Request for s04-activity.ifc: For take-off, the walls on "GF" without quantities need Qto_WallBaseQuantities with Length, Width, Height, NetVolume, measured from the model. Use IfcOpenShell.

First a look at what the model holds.

```python
import ifcopenshell
import ifcopenshell.util.element
import ifcopenshell.util.unit

model = ifcopenshell.open("s04-activity.ifc")
print(model.schema)
for unit_type in ("LENGTHUNIT", "AREAUNIT", "VOLUMEUNIT"):
    print(unit_type, ifcopenshell.util.unit.calculate_unit_scale(model, unit_type))
storey = next(s for s in model.by_type("IfcBuildingStorey") if s.Name == "GF")
walls = [e for e in ifcopenshell.util.element.get_decomposition(storey) if e.is_a("IfcWall")]
for e in sorted(walls, key=lambda e: e.id()):
    print(e.id(), e.is_a(), e.Name, list(ifcopenshell.util.element.get_psets(e, qtos_only=True)), sep=" | ")
```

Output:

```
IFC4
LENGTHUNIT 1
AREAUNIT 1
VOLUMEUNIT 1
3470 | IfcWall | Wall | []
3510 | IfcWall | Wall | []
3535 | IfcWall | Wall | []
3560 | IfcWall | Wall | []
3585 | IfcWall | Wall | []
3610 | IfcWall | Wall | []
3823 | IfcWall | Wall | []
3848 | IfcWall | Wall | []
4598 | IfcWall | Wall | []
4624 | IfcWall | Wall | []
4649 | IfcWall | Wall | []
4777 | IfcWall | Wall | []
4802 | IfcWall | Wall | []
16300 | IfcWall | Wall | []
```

```python
import ifcopenshell
import ifcopenshell.api.pset
import ifcopenshell.geom
import ifcopenshell.util.element
import ifcopenshell.util.shape
import ifcopenshell.util.unit

model = ifcopenshell.open("s04-activity.ifc")
unit_scale = ifcopenshell.util.unit.calculate_unit_scale(model)
volume_scale = ifcopenshell.util.unit.calculate_unit_scale(model, "VOLUMEUNIT")
settings = ifcopenshell.geom.settings()

storey = next(s for s in model.by_type("IfcBuildingStorey") if s.Name == "GF")
walls = [e for e in ifcopenshell.util.element.get_decomposition(storey) if e.is_a("IfcWall")]

for e in sorted(walls, key=lambda e: e.id()):
    if ifcopenshell.util.element.get_psets(e, qtos_only=True, should_inherit=False):
        continue
    # Geometry comes back in metres, in the element's own axes.
    shape = ifcopenshell.geom.create_shape(settings, e)
    values = {
        "Length": ifcopenshell.util.shape.get_x(shape.geometry) / unit_scale,
        "Width": ifcopenshell.util.shape.get_y(shape.geometry) / unit_scale,
        "Height": ifcopenshell.util.shape.get_z(shape.geometry) / unit_scale,
        "NetVolume": ifcopenshell.util.shape.get_volume(shape.geometry) / volume_scale,
    }
    qto = ifcopenshell.api.pset.add_qto(model, product=e, name="Qto_WallBaseQuantities")
    ifcopenshell.api.pset.edit_qto(model, qto=qto, properties=values)
    print(e.id(), {k: round(v, 3) for k, v in values.items()})

model.write("s04-activity_updated.ifc")
```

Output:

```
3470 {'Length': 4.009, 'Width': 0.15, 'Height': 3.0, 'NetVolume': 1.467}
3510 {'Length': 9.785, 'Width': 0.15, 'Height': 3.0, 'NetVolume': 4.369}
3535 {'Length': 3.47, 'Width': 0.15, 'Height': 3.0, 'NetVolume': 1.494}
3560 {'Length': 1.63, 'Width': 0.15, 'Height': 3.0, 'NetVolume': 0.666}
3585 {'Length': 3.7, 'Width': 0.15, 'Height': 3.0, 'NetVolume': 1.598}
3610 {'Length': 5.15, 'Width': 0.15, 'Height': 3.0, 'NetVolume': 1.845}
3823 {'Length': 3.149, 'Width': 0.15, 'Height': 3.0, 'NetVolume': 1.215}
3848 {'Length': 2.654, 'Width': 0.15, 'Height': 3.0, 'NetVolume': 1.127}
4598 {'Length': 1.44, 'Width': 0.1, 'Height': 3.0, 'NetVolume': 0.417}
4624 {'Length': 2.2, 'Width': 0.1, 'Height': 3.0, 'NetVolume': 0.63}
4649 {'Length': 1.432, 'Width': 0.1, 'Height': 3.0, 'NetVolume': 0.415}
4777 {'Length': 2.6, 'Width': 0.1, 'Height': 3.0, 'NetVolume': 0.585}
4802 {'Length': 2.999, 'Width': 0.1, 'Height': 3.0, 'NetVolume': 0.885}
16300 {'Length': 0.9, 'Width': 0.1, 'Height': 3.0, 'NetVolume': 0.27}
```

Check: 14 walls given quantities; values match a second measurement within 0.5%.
